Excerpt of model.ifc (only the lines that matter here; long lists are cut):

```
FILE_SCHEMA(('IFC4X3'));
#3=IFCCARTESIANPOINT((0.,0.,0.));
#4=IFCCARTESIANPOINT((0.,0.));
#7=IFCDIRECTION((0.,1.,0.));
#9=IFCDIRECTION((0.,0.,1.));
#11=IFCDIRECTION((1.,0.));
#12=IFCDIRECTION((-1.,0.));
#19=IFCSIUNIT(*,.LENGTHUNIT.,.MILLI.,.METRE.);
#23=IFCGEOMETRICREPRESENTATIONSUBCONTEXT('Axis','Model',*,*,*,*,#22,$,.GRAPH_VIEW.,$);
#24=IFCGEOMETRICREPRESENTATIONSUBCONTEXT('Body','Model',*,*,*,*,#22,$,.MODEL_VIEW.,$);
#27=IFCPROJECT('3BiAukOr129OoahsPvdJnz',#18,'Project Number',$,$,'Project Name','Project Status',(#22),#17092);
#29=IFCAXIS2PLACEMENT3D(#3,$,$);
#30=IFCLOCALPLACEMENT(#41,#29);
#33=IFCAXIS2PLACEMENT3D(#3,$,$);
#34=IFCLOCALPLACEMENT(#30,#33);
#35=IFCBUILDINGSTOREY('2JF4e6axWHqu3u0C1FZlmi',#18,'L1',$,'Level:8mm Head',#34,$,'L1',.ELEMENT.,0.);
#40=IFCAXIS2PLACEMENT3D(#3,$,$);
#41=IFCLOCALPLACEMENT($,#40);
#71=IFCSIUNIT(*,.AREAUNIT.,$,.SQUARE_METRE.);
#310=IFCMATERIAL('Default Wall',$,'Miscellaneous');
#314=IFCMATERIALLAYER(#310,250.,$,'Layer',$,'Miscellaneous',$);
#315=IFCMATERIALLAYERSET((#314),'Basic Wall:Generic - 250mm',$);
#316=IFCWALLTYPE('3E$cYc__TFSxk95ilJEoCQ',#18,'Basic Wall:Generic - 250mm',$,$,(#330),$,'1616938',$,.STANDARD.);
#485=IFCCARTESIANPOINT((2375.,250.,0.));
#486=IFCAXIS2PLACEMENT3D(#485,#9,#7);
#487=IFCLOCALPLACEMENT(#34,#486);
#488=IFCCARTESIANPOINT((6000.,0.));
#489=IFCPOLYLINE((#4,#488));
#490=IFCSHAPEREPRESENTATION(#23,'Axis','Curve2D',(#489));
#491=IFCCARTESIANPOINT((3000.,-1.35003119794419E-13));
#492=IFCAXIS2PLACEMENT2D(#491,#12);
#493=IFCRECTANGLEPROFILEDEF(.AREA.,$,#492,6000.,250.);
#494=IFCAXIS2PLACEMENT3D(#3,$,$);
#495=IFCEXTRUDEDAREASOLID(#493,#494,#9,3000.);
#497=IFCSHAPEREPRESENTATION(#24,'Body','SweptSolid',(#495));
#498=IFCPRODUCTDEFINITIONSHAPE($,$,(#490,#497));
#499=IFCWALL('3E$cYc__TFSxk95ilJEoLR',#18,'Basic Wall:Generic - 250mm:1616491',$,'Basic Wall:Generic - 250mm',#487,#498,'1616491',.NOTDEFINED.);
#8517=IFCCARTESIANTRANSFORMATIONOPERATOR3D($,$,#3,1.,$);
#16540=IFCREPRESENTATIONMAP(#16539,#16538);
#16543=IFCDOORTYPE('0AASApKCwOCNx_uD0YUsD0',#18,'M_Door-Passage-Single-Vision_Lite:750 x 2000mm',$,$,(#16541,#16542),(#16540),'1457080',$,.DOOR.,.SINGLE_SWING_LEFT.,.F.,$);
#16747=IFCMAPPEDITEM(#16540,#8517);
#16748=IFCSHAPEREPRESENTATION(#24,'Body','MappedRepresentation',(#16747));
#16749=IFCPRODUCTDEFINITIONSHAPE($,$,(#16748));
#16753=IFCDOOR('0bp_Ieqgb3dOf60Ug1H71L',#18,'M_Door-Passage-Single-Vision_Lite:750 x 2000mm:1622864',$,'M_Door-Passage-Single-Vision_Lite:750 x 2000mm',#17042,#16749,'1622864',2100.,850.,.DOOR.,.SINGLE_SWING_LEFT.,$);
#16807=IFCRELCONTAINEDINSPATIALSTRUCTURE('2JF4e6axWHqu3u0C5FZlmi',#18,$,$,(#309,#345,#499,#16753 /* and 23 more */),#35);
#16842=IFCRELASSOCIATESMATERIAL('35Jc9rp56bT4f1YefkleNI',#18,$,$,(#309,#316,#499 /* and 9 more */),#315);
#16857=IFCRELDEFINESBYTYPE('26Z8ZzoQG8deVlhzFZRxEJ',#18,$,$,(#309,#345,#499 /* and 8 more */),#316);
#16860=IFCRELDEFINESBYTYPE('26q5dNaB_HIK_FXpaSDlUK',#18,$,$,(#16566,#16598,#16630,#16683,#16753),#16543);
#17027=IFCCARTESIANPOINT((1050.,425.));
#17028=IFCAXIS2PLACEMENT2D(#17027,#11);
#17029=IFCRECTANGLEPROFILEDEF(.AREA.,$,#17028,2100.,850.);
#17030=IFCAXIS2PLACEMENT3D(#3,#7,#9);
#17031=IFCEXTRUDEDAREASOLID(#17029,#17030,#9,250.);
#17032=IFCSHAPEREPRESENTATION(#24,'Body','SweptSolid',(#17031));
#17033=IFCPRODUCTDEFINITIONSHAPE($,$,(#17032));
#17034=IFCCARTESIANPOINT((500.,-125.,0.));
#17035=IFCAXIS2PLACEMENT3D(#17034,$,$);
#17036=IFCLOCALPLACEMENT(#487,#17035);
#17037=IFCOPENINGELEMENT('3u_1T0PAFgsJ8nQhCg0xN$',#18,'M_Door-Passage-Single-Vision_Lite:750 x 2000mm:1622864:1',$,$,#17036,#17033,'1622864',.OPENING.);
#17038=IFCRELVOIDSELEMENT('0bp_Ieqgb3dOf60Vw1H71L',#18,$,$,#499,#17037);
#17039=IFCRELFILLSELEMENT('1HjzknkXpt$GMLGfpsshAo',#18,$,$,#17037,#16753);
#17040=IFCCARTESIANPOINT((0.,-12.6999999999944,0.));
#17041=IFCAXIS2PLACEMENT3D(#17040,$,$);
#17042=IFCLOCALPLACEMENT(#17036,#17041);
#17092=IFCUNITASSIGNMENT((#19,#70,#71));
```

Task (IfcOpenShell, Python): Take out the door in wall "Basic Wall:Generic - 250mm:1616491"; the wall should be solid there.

```python
import ifcopenshell
import ifcopenshell.api.feature
import ifcopenshell.api.root
import ifcopenshell.geom
import ifcopenshell.util.shape

model = ifcopenshell.open("model.ifc")
settings = ifcopenshell.geom.settings()


def volume(element):
    """Net volume in cubic metres, openings subtracted."""
    shape = ifcopenshell.geom.create_shape(settings, element)
    return ifcopenshell.util.shape.get_volume(shape.geometry)


door = model.by_id(16753)
opening = door.FillsVoids[0].RelatingOpeningElement
wall = opening.VoidsElements[0].RelatingBuildingElement
before = volume(wall)

ifcopenshell.api.root.remove_product(model, product=door)
ifcopenshell.api.feature.remove_feature(model, feature=opening)

after = volume(wall)

print(f"wall volume {before:.3f} -> {after:.3f} m3")

model.write("model_updated.ifc")
```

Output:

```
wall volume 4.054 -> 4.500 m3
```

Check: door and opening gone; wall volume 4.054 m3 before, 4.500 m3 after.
